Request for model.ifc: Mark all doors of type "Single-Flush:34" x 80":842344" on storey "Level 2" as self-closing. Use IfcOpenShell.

First a look at what the model holds.

```python
import ifcopenshell
import ifcopenshell.util.element

model = ifcopenshell.open("model.ifc")
print(model.schema)
storey = next(s for s in model.by_type("IfcBuildingStorey") if s.Name == "Level 2")
doors = [e for e in ifcopenshell.util.element.get_decomposition(storey) if e.is_a("IfcDoor")]
seen = {}
for e in doors:
    element_type = ifcopenshell.util.element.get_type(e)
    key = (element_type.Name if element_type != e and element_type else None, ifcopenshell.util.element.get_pset(e, "Pset_DoorCommon", "SelfClosing"))
    seen[key] = seen.get(key, 0) + 1
for (name, value), count in sorted(seen.items(), key=str):
    print(count, "x", name, "|", value)
```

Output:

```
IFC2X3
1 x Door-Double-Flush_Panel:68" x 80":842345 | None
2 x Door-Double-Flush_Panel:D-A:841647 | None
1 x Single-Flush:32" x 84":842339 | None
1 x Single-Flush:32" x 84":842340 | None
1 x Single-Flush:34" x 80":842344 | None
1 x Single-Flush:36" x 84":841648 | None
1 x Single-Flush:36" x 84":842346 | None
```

```python
import ifcopenshell
import ifcopenshell.api.pset
import ifcopenshell.util.element

model = ifcopenshell.open("model.ifc")

storey = next(s for s in model.by_type("IfcBuildingStorey") if s.Name == "Level 2")
doors = [e for e in ifcopenshell.util.element.get_decomposition(storey) if e.is_a("IfcDoor")]

count = 0
for e in doors:
    element_type = ifcopenshell.util.element.get_type(e)
    if element_type in (None, e) or element_type.Name != 'Single-Flush:34" x 80":842344':
        continue
    # add_pset returns the element's existing set when there is one.
    pset = ifcopenshell.api.pset.add_pset(model, product=e, name="Pset_DoorCommon")
    ifcopenshell.api.pset.edit_pset(model, pset=pset, properties={"SelfClosing": True})
    count += 1

print(count, "doors updated")

model.write("model_edited.ifc")
```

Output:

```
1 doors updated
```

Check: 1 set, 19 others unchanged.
